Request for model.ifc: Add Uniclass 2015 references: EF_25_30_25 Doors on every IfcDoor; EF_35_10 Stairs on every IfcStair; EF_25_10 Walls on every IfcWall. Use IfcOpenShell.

First a look at what the model holds.

```python
import ifcopenshell

model = ifcopenshell.open("model.ifc")
print(model.schema)
print("classifications:", [c.Name for c in model.by_type("IfcClassification")])
for ifc_class in ("IfcDoor", "IfcRoof", "IfcStair", "IfcWall", "IfcWindow"):
    print(ifc_class, len(model.by_type(ifc_class)))
```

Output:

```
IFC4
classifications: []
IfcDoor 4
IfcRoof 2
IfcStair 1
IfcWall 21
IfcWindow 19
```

```python
import ifcopenshell
import ifcopenshell.api.classification

model = ifcopenshell.open("model.ifc")

system = ifcopenshell.api.classification.add_classification(model, classification="Uniclass 2015")

codes = {
    "IfcDoor": ("EF_25_30_25", "Doors"),
    "IfcStair": ("EF_35_10", "Stairs"),
    "IfcWall": ("EF_25_10", "Walls"),
}
for ifc_class, (code, name) in codes.items():
    products = model.by_type(ifc_class)
    ifcopenshell.api.classification.add_reference(
        model, products=products, classification=system, identification=code, name=name
    )
    print(code, len(products))

model.write("model_v2.ifc")
```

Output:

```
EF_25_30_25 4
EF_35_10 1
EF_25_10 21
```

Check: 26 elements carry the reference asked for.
